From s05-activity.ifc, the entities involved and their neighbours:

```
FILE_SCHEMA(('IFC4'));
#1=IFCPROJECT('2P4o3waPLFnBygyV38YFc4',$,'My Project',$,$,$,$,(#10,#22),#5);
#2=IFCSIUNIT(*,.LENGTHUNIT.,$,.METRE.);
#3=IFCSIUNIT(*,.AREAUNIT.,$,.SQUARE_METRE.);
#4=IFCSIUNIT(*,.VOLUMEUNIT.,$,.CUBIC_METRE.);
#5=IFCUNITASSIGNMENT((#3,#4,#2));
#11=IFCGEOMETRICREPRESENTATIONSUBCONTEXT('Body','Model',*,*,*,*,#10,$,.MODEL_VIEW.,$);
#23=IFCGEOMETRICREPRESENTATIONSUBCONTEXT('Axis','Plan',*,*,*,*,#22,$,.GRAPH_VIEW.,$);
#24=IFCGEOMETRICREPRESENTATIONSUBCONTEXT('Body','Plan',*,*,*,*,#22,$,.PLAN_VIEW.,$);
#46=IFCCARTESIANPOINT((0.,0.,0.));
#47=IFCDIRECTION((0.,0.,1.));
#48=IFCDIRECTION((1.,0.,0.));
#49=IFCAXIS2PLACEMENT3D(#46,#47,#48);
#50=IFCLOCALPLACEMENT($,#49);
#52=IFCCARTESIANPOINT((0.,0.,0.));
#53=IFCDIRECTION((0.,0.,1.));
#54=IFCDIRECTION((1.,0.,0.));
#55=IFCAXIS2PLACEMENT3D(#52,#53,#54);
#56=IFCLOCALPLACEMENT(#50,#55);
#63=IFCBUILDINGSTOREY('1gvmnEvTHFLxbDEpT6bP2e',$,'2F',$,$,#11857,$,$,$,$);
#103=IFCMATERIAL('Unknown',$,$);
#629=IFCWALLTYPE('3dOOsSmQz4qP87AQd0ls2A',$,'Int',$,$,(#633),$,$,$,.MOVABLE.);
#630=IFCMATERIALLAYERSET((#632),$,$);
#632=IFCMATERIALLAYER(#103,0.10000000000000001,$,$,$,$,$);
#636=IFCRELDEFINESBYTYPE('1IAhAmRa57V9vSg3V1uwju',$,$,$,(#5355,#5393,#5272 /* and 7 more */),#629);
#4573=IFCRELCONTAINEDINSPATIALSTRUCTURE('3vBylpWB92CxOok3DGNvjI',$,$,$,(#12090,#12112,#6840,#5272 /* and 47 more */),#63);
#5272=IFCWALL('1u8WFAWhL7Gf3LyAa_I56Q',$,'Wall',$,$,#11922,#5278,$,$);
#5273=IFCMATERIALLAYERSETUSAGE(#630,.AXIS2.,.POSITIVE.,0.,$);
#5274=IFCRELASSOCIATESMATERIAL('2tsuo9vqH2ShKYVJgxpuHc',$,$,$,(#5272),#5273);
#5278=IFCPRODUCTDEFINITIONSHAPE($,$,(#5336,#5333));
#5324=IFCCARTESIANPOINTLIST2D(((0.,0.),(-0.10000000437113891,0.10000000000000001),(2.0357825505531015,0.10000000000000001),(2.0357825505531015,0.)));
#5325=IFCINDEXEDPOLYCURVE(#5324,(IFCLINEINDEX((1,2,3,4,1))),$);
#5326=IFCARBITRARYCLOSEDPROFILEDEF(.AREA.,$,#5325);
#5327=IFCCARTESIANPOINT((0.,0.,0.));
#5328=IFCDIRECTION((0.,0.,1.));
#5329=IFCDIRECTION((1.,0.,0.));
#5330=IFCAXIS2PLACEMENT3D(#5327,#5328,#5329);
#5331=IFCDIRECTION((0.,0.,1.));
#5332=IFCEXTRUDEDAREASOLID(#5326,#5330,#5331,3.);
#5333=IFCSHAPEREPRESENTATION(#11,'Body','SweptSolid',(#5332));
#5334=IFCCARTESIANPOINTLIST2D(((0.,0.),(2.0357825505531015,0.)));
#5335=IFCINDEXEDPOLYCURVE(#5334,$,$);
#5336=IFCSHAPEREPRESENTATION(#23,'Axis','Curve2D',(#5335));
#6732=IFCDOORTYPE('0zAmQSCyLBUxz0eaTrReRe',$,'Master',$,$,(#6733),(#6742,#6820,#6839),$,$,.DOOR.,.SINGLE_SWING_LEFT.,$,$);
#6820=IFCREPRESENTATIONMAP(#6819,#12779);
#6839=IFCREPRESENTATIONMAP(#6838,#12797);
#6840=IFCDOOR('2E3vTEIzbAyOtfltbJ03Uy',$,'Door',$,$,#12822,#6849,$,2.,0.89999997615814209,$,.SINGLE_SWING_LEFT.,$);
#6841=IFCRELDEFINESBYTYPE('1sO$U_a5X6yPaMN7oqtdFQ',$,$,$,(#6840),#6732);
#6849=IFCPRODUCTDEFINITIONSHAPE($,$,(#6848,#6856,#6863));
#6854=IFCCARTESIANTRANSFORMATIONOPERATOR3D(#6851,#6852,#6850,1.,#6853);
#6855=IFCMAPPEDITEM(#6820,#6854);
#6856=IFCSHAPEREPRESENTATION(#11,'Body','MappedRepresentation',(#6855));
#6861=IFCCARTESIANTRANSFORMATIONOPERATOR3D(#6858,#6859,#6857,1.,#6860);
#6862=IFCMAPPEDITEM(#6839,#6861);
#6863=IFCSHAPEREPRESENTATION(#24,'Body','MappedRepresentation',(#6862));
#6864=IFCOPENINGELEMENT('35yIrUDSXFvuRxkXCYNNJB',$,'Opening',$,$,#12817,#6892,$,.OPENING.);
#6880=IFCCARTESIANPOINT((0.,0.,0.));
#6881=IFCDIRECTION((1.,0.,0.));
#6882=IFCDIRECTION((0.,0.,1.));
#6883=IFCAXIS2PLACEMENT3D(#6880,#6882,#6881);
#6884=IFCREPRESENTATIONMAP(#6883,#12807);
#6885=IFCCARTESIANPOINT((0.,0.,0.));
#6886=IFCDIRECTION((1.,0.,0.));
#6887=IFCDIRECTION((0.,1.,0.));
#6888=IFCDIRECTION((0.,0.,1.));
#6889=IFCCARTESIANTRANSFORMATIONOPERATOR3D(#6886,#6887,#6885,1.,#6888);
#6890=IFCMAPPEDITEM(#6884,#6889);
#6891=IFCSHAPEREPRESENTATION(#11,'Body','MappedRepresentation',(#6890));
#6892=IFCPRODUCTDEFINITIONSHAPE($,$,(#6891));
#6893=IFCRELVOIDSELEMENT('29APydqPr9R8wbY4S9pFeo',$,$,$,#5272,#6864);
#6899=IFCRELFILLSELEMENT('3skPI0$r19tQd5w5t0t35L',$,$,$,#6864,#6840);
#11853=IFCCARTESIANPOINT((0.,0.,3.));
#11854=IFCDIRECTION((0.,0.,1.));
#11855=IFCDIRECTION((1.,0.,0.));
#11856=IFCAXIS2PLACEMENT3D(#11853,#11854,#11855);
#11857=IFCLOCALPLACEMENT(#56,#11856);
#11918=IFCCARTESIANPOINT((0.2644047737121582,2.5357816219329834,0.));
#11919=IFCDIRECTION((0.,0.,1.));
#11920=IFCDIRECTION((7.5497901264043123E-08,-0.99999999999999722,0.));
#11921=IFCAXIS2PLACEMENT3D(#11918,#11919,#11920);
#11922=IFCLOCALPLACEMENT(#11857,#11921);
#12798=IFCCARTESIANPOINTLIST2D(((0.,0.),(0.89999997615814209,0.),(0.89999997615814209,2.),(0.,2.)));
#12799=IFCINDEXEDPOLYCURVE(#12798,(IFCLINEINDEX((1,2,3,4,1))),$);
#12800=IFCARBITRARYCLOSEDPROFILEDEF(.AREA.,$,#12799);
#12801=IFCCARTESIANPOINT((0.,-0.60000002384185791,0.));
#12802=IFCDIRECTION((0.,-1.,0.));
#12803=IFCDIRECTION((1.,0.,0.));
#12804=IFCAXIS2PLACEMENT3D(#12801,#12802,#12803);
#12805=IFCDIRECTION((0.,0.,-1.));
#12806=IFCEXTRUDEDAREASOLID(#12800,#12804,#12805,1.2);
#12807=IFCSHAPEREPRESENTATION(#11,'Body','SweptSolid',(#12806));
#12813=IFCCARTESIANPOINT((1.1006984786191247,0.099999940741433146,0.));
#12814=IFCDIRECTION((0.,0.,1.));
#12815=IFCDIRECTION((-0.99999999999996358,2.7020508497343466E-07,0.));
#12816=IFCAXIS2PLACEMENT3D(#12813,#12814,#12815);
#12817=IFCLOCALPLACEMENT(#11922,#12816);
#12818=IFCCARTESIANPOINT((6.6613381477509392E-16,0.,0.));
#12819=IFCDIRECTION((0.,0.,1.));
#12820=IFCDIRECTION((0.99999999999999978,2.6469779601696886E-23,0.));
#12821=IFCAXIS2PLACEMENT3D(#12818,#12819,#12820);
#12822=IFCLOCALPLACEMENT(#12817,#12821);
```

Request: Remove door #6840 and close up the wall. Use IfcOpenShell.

```python
import ifcopenshell
import ifcopenshell.api.feature
import ifcopenshell.api.root
import ifcopenshell.geom
import ifcopenshell.util.shape

model = ifcopenshell.open("s05-activity.ifc")
settings = ifcopenshell.geom.settings()


def volume(element):
    """Net volume in cubic metres, openings subtracted."""
    shape = ifcopenshell.geom.create_shape(settings, element)
    return ifcopenshell.util.shape.get_volume(shape.geometry)


door = model.by_id(6840)
opening = door.FillsVoids[0].RelatingOpeningElement
wall = opening.VoidsElements[0].RelatingBuildingElement
before = volume(wall)

ifcopenshell.api.root.remove_product(model, product=door)
ifcopenshell.api.feature.remove_feature(model, feature=opening)

after = volume(wall)

print(f"wall volume {before:.3f} -> {after:.3f} m3")

model.write("s05-activity_edited.ifc")
```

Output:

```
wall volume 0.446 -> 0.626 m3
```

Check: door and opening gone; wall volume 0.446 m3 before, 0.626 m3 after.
